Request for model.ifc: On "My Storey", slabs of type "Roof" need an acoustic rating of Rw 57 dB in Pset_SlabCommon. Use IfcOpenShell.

First a look at what the model holds.

```python
import ifcopenshell
import ifcopenshell.util.element

model = ifcopenshell.open("model.ifc")
print(model.schema)
storey = next(s for s in model.by_type("IfcBuildingStorey") if s.Name == "My Storey")
slabs = [e for e in ifcopenshell.util.element.get_decomposition(storey) if e.is_a("IfcSlab")]
seen = {}
for e in slabs:
    element_type = ifcopenshell.util.element.get_type(e)
    key = (element_type.Name if element_type != e and element_type else None, ifcopenshell.util.element.get_pset(e, "Pset_SlabCommon", "AcousticRating"))
    seen[key] = seen.get(key, 0) + 1
for (name, value), count in sorted(seen.items(), key=str):
    print(count, "x", name, "|", value)
```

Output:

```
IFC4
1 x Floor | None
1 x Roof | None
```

```python
import ifcopenshell
import ifcopenshell.api.pset
import ifcopenshell.util.element

model = ifcopenshell.open("model.ifc")

storey = next(s for s in model.by_type("IfcBuildingStorey") if s.Name == "My Storey")
slabs = [e for e in ifcopenshell.util.element.get_decomposition(storey) if e.is_a("IfcSlab")]

count = 0
for e in slabs:
    element_type = ifcopenshell.util.element.get_type(e)
    if element_type in (None, e) or element_type.Name != "Roof":
        continue
    # add_pset returns the element's existing set when there is one.
    pset = ifcopenshell.api.pset.add_pset(model, product=e, name="Pset_SlabCommon")
    ifcopenshell.api.pset.edit_pset(model, pset=pset, properties={"AcousticRating": "Rw 57 dB"})
    count += 1

print(count, "slabs updated")

model.write("model_edited.ifc")
```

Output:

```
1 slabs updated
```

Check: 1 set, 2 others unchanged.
